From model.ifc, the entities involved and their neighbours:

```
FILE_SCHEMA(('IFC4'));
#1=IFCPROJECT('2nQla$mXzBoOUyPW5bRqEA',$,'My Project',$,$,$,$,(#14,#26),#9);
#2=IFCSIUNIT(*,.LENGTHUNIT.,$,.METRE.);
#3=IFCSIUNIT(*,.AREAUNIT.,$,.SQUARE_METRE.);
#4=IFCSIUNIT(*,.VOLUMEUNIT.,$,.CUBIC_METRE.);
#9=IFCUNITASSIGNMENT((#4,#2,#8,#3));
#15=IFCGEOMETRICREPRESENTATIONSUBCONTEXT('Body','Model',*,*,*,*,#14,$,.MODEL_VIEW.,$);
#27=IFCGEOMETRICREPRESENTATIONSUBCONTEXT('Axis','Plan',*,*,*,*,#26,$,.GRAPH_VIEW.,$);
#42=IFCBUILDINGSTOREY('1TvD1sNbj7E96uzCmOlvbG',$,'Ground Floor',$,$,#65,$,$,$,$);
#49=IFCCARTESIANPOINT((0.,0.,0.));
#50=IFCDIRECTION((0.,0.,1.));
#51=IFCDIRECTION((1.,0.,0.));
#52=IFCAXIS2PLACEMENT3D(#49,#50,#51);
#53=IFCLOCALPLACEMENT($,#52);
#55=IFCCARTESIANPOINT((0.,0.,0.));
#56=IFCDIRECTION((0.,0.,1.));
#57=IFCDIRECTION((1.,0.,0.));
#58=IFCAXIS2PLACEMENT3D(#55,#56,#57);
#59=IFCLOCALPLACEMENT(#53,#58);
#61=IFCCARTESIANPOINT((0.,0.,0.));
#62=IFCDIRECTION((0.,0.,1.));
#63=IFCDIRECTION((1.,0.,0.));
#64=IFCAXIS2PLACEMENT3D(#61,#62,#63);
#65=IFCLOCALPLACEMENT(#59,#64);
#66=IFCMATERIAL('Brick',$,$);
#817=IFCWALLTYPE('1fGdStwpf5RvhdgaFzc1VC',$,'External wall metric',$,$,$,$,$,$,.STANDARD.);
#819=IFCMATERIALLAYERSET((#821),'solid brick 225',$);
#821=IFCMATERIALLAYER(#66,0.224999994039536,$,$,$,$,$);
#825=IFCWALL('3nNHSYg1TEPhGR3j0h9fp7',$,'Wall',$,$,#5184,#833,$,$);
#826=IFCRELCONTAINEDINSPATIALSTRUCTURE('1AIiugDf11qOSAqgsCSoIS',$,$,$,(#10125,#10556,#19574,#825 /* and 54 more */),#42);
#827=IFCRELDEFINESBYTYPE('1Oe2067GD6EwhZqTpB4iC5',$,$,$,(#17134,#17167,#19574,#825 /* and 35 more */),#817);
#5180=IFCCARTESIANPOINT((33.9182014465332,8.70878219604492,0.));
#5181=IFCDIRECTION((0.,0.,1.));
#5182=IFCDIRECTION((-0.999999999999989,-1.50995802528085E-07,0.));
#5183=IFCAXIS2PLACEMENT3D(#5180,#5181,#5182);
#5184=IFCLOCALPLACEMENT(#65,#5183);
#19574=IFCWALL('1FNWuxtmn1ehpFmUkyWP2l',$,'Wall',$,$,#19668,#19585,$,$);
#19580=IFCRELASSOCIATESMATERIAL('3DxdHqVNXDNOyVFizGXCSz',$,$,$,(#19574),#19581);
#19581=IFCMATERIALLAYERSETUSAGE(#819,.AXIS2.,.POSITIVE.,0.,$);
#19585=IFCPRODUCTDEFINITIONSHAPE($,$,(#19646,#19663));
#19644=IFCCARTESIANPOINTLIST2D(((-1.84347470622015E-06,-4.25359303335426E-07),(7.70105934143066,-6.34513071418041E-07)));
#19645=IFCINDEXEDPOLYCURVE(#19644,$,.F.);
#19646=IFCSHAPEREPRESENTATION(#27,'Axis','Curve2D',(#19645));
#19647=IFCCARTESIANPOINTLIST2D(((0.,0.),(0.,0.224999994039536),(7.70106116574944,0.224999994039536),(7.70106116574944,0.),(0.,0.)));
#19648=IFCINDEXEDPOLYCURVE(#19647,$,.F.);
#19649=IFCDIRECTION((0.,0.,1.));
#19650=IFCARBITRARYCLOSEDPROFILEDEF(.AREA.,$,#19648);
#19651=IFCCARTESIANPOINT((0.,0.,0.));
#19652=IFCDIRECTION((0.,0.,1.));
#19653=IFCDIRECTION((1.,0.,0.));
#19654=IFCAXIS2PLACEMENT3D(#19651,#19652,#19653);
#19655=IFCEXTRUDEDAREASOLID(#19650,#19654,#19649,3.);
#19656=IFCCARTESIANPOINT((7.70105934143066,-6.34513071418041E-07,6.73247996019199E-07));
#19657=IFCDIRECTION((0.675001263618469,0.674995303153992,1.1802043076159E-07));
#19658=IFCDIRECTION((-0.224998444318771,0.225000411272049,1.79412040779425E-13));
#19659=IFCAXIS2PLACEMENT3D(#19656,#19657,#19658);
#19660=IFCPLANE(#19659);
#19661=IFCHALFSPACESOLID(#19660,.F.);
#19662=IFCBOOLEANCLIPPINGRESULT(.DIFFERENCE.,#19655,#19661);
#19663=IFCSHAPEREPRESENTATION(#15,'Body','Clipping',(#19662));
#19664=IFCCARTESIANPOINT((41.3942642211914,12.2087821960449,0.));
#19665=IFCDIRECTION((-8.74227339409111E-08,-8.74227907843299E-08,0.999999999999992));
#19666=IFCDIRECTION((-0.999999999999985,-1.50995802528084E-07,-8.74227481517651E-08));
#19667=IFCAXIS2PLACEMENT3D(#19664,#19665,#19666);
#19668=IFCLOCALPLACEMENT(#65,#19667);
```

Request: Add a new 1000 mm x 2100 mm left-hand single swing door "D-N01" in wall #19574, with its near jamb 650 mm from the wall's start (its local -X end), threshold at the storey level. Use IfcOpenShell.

```python
import numpy as np
import ifcopenshell
import ifcopenshell.api.feature
import ifcopenshell.api.geometry
import ifcopenshell.api.root
import ifcopenshell.api.spatial
import ifcopenshell.geom
import ifcopenshell.util.element
import ifcopenshell.util.placement
import ifcopenshell.util.representation
import ifcopenshell.util.shape
import ifcopenshell.util.unit

model = ifcopenshell.open("model.ifc")
unit_scale = ifcopenshell.util.unit.calculate_unit_scale(model)
settings = ifcopenshell.geom.settings()


def volume(element):
    """Net volume in cubic metres, openings subtracted."""
    shape = ifcopenshell.geom.create_shape(settings, element)
    return ifcopenshell.util.shape.get_volume(shape.geometry)


wall = model.by_guid("1FNWuxtmn1ehpFmUkyWP2l")
storey = ifcopenshell.util.element.get_container(wall, ifc_class="IfcBuildingStorey")
context = ifcopenshell.util.representation.get_context(model, "Model", "Body", "MODEL_VIEW")
before = volume(wall)

width, height, from_end, sill = 1, 2.1, 0.65, 0.0  # metres

# The wall runs along its own X axis, and the end named is its -X end.
wall_shape = ifcopenshell.geom.create_shape(settings, wall)
x, y, z = ifcopenshell.util.shape.get_vertices(wall_shape.geometry).T
start = x.min() + from_end
face, thickness = float(y.min()), float(y.max() - y.min())
wall_matrix = ifcopenshell.util.placement.get_local_placement(wall.ObjectPlacement)
level = ifcopenshell.util.placement.get_local_placement(storey.ObjectPlacement)[2, 3]


def in_wall(x, y):
    """Placement at x, y metres in the wall's axes, at sill height."""
    matrix = wall_matrix.copy()
    matrix[:, 3] = wall_matrix @ np.array([x / unit_scale, y / unit_scale, 0.0, 1.0])
    matrix[2, 3] = level + sill / unit_scale
    return matrix


# Opening: a box that overshoots both wall faces by 50 mm.
opening = ifcopenshell.api.root.create_entity(model, ifc_class="IfcOpeningElement", predefined_type="OPENING")
box = ifcopenshell.api.geometry.add_wall_representation(
    model, context=context, length=width, height=height, thickness=thickness + 0.1
)
ifcopenshell.api.geometry.assign_representation(model, product=opening, representation=box)
ifcopenshell.api.geometry.edit_object_placement(model, product=opening, matrix=in_wall(start, face - 0.05), is_si=False)
ifcopenshell.api.feature.add_feature(model, feature=opening, element=wall)

door = ifcopenshell.api.root.create_entity(model, ifc_class="IfcDoor", name="D-N01", predefined_type="DOOR")
door.OverallWidth, door.OverallHeight = width / unit_scale, height / unit_scale
door.OperationType = "SINGLE_SWING_LEFT"
body = ifcopenshell.api.geometry.add_door_representation(
    model,
    context=context,
    overall_width=door.OverallWidth,
    overall_height=door.OverallHeight,
    operation_type="SINGLE_SWING_LEFT",
    lining_properties={"LiningDepth": thickness / unit_scale, "ThresholdDepth": thickness / unit_scale},
)
ifcopenshell.api.geometry.assign_representation(model, product=door, representation=body)
ifcopenshell.api.spatial.assign_container(model, products=[door], relating_structure=storey)
ifcopenshell.api.feature.add_filling(model, opening=opening, element=door)

# The lining spans the wall, so the door starts at the wall face.
ifcopenshell.api.geometry.edit_object_placement(model, product=door, matrix=in_wall(start, face), is_si=False)

after = volume(wall)

print(f"wall volume {before:.3f} -> {after:.3f} m3")

model.write("model_rev.ifc")
```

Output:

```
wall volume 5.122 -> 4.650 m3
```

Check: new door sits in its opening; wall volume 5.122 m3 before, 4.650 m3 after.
